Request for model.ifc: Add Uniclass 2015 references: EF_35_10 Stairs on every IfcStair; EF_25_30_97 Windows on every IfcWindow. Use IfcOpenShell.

First a look at what the model holds.

```python
import ifcopenshell

model = ifcopenshell.open("model.ifc")
print(model.schema)
print("classifications:", [c.Name for c in model.by_type("IfcClassification")])
for ifc_class in ("IfcDoor", "IfcRoof", "IfcStair", "IfcWall", "IfcWindow"):
    print(ifc_class, len(model.by_type(ifc_class)))
```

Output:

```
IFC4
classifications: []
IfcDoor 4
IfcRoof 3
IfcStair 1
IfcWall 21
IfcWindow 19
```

```python
import ifcopenshell
import ifcopenshell.api.classification

model = ifcopenshell.open("model.ifc")

system = ifcopenshell.api.classification.add_classification(model, classification="Uniclass 2015")

codes = {
    "IfcStair": ("EF_35_10", "Stairs"),
    "IfcWindow": ("EF_25_30_97", "Windows"),
}
for ifc_class, (code, name) in codes.items():
    products = model.by_type(ifc_class)
    ifcopenshell.api.classification.add_reference(
        model, products=products, classification=system, identification=code, name=name
    )
    print(code, len(products))

model.write("model_updated.ifc")
```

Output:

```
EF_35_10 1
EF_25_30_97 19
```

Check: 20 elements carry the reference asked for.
